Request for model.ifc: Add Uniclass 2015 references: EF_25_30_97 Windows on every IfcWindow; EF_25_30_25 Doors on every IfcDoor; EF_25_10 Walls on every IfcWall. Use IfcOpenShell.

First a look at what the model holds.

```python
import ifcopenshell

model = ifcopenshell.open("model.ifc")
print(model.schema)
print("classifications:", [c.Name for c in model.by_type("IfcClassification")])
for ifc_class in ("IfcDoor", "IfcRoof", "IfcStair", "IfcWall", "IfcWindow"):
    print(ifc_class, len(model.by_type(ifc_class)))
```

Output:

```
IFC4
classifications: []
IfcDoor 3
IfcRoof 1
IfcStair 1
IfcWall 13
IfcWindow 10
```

```python
import ifcopenshell
import ifcopenshell.api.classification

model = ifcopenshell.open("model.ifc")

system = ifcopenshell.api.classification.add_classification(model, classification="Uniclass 2015")

codes = {
    "IfcWindow": ("EF_25_30_97", "Windows"),
    "IfcDoor": ("EF_25_30_25", "Doors"),
    "IfcWall": ("EF_25_10", "Walls"),
}
for ifc_class, (code, name) in codes.items():
    products = model.by_type(ifc_class)
    ifcopenshell.api.classification.add_reference(
        model, products=products, classification=system, identification=code, name=name
    )
    print(code, len(products))

model.write("model_edited.ifc")
```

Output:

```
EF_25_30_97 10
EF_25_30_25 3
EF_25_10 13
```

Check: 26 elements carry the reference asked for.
